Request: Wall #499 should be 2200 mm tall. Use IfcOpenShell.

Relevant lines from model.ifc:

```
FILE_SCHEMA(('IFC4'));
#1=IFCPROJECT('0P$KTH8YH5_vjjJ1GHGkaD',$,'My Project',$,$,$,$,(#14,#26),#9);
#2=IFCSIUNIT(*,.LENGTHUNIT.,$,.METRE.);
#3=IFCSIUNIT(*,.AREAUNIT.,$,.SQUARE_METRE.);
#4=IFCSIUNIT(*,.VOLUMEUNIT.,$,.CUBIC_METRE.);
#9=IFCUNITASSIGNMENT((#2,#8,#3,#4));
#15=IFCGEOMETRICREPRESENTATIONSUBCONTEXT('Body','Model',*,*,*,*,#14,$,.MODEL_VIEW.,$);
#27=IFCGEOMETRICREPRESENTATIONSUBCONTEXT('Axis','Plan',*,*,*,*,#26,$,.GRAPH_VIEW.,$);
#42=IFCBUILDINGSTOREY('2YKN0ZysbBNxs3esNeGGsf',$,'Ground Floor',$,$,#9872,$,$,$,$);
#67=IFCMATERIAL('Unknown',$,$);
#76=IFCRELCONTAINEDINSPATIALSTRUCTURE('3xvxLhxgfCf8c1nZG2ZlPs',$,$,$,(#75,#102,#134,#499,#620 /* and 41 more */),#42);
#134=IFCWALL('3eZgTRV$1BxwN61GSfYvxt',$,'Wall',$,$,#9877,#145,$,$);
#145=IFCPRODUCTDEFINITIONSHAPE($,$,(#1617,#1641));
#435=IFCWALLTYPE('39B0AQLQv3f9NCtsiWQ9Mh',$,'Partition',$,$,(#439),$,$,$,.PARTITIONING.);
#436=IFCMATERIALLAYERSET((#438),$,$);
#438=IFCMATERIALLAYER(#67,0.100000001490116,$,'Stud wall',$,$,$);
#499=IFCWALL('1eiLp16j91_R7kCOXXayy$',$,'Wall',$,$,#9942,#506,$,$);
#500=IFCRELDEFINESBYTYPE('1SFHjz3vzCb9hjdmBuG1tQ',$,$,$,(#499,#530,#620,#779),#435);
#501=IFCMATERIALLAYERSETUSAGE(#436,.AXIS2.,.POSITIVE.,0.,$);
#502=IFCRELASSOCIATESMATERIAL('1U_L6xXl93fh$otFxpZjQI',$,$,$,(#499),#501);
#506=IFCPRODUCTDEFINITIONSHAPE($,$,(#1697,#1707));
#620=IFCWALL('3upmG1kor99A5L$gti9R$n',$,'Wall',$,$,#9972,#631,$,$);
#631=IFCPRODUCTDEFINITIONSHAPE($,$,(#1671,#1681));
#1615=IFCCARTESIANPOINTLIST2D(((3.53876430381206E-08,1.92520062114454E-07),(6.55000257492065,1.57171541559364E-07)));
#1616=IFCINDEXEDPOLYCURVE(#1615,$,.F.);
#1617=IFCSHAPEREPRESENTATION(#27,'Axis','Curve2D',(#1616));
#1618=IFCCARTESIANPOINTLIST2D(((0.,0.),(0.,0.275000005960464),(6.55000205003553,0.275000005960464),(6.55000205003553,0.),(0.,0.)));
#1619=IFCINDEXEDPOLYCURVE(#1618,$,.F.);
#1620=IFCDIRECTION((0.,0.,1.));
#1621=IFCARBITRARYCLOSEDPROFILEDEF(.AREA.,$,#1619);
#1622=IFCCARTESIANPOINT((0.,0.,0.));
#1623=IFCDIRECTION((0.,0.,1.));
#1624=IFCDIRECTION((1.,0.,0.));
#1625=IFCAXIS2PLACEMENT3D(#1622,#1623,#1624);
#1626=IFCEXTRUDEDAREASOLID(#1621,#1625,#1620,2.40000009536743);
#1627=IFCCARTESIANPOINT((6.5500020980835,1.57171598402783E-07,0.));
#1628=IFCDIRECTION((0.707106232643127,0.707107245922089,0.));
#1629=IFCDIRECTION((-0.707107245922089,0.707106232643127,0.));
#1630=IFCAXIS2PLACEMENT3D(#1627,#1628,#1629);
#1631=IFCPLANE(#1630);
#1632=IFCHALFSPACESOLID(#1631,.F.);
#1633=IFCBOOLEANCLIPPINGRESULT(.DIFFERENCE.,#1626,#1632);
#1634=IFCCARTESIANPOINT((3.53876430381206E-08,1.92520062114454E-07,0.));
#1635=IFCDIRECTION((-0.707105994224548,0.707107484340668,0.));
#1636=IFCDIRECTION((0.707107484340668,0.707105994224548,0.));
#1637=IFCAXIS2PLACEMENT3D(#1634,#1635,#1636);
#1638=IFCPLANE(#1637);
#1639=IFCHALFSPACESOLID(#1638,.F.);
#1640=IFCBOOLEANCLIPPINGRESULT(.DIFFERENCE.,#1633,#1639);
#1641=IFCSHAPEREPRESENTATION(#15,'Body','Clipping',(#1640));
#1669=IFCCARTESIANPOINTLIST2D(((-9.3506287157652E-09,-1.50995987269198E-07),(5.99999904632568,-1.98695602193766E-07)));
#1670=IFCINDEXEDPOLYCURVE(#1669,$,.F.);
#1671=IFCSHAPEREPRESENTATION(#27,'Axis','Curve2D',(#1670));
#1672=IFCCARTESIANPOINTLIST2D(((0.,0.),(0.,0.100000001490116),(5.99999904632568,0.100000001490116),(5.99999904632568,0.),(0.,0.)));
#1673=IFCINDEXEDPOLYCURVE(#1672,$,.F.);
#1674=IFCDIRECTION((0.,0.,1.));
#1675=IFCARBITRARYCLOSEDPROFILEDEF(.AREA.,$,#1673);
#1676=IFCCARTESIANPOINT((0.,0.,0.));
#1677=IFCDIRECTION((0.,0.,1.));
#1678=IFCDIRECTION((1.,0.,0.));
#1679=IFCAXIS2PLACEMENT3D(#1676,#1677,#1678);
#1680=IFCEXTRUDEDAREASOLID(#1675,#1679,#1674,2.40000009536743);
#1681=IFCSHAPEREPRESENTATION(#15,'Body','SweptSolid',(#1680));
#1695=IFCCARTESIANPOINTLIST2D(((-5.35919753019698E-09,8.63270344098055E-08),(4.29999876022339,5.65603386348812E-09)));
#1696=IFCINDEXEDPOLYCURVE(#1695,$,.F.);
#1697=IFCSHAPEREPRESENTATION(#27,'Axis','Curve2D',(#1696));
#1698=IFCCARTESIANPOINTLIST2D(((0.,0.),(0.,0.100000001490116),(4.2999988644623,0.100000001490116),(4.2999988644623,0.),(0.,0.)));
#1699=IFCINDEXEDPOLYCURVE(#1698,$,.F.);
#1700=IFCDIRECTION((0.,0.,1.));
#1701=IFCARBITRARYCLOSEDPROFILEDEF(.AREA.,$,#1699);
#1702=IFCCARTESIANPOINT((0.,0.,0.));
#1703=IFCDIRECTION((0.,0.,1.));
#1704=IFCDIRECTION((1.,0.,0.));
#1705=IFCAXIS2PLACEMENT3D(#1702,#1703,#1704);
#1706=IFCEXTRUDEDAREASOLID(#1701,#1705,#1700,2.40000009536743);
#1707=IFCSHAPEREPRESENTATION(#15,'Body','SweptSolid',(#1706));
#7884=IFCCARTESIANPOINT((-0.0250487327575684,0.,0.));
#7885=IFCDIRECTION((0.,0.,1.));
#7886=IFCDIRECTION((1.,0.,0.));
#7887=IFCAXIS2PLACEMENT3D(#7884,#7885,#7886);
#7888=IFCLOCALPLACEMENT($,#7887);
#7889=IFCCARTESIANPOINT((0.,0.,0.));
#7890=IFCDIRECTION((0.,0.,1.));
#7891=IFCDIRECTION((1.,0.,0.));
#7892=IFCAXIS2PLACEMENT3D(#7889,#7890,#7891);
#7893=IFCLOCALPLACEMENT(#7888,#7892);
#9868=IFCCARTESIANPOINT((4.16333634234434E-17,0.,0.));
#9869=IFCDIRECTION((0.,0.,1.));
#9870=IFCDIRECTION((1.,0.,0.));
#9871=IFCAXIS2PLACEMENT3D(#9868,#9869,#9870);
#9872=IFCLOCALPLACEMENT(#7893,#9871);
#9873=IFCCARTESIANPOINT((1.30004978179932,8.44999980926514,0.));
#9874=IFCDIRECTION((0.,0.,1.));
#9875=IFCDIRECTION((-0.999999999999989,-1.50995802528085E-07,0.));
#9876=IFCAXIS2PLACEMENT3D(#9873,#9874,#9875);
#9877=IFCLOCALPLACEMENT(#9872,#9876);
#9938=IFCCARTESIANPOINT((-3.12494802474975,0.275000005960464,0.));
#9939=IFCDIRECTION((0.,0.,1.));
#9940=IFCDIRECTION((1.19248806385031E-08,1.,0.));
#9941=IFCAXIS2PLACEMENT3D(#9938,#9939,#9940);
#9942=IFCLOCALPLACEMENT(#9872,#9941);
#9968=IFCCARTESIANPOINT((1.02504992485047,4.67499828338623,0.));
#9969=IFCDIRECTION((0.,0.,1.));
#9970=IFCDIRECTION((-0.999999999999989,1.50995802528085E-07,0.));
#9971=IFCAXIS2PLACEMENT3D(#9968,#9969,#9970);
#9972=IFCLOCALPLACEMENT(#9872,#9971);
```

```python
import ifcopenshell
import ifcopenshell.geom
import ifcopenshell.util.representation
import ifcopenshell.util.shape
import ifcopenshell.util.unit

model = ifcopenshell.open("model.ifc")
unit_scale = ifcopenshell.util.unit.calculate_unit_scale(model)
settings = ifcopenshell.geom.settings()


def volume(element):
    """Net volume in cubic metres, openings subtracted."""
    shape = ifcopenshell.geom.create_shape(settings, element)
    return ifcopenshell.util.shape.get_volume(shape.geometry)


wall = model.by_guid("1eiLp16j91_R7kCOXXayy$")
before = volume(wall)

body = ifcopenshell.util.representation.get_representation(wall, "Model", "Body")
solid = body.Items[0]
old_height = solid.Depth
solid.Depth = 2.2 / unit_scale
after = volume(wall)

print(f"height {old_height:g} -> {solid.Depth:g}, volume {before:.3f} -> {after:.3f} m3")

model.write("model_edited.ifc")
```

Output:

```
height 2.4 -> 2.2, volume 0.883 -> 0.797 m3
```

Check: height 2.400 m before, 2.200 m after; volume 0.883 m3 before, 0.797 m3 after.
